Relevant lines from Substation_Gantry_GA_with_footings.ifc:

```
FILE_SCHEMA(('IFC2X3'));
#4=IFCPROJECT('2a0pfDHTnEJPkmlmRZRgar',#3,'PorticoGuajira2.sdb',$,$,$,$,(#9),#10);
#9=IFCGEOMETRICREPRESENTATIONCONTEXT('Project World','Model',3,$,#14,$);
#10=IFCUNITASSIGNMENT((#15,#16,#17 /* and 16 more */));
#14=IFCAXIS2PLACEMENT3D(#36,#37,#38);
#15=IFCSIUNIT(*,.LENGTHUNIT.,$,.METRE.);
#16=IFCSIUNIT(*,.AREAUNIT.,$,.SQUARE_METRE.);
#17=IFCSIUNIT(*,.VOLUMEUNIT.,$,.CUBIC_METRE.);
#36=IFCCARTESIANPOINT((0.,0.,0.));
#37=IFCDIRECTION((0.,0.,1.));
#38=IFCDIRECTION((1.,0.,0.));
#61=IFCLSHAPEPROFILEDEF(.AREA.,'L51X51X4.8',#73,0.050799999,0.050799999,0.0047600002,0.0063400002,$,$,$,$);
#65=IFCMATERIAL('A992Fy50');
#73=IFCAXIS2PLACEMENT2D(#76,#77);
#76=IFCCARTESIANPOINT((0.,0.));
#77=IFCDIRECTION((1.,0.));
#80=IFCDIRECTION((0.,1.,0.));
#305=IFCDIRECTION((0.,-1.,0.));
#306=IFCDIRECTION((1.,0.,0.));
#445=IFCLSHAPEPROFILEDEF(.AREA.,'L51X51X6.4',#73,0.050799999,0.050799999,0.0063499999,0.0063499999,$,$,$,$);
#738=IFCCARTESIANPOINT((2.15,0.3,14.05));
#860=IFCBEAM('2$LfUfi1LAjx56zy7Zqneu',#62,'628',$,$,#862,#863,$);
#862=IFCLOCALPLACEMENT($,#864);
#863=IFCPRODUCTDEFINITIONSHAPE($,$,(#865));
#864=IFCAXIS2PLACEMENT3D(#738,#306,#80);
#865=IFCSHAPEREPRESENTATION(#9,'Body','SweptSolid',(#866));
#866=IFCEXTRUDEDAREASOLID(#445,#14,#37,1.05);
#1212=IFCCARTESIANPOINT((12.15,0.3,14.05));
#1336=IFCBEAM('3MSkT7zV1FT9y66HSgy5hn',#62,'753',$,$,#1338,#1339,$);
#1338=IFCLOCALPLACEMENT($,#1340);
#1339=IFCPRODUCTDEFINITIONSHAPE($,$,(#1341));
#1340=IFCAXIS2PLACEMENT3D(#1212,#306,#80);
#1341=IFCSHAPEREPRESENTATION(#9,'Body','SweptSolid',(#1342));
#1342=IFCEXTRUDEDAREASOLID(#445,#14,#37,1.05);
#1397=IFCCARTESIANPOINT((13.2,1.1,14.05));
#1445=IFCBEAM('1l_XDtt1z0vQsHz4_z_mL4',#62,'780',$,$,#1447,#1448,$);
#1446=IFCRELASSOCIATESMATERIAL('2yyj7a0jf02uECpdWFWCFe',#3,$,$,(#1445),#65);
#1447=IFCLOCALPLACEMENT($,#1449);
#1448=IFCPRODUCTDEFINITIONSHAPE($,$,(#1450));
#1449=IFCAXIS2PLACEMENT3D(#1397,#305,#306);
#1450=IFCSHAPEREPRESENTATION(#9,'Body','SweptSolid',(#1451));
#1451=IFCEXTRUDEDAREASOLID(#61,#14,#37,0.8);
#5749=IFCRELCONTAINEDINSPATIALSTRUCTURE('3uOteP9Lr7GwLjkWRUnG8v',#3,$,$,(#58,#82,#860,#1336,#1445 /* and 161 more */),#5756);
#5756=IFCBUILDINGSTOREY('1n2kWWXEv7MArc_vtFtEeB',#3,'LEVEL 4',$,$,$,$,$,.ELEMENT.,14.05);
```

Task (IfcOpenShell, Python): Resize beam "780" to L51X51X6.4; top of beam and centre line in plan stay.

```python
import ifcopenshell
import ifcopenshell.util.element

model = ifcopenshell.open("Substation_Gantry_GA_with_footings.ifc")

member = model.by_guid("1l_XDtt1z0vQsHz4_z_mL4")
source = next(p for p in model.by_type("IfcLShapeProfileDef") if p.ProfileName == "L51X51X6.4")

body = next(r for r in member.Representation.Representations if r.RepresentationIdentifier == "Body")
solid = body.Items[0]
old_profile = solid.SweptArea

# Copy the section's sizes but keep this member's own profile position.
profile = ifcopenshell.util.element.copy(model, source)
# Profiles are centred, so shift by half the change in depth to hold the top.
shift = (old_profile.Depth - profile.Depth) / 2
x, y = old_profile.Position.Location.Coordinates
up = (0.0, 1.0)  # upwards, in the solid's own plane
location = model.createIfcCartesianPoint((x + up[0] * shift, y + up[1] * shift))
profile.Position = model.createIfcAxis2Placement2D(location, old_profile.Position.RefDirection)
solid.SweptArea = profile
if not model.get_total_inverses(old_profile):
    ifcopenshell.util.element.remove_deep2(model, old_profile)

print(solid.SweptArea)

model.write("Substation_Gantry_GA_with_footings_edited.ifc")
```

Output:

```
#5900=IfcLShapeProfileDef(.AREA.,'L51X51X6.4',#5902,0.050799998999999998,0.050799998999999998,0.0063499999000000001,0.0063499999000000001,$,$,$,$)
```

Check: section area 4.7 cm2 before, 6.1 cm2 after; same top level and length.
